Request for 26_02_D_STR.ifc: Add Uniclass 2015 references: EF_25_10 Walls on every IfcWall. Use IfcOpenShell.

First a look at what the model holds.

```python
import ifcopenshell

model = ifcopenshell.open("26_02_D_STR.ifc")
print(model.schema)
print("classifications:", [c.Name for c in model.by_type("IfcClassification")])
for ifc_class in ("IfcDoor", "IfcRoof", "IfcStair", "IfcWall", "IfcWindow"):
    print(ifc_class, len(model.by_type(ifc_class)))
```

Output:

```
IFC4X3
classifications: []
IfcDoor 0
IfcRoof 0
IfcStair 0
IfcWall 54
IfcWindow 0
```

```python
import ifcopenshell
import ifcopenshell.api.classification

model = ifcopenshell.open("26_02_D_STR.ifc")

system = ifcopenshell.api.classification.add_classification(model, classification="Uniclass 2015")

codes = {
    "IfcWall": ("EF_25_10", "Walls"),
}
for ifc_class, (code, name) in codes.items():
    products = model.by_type(ifc_class)
    ifcopenshell.api.classification.add_reference(
        model, products=products, classification=system, identification=code, name=name
    )
    print(code, len(products))

model.write("26_02_D_STR_v2.ifc")
```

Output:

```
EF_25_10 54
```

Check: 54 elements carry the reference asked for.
